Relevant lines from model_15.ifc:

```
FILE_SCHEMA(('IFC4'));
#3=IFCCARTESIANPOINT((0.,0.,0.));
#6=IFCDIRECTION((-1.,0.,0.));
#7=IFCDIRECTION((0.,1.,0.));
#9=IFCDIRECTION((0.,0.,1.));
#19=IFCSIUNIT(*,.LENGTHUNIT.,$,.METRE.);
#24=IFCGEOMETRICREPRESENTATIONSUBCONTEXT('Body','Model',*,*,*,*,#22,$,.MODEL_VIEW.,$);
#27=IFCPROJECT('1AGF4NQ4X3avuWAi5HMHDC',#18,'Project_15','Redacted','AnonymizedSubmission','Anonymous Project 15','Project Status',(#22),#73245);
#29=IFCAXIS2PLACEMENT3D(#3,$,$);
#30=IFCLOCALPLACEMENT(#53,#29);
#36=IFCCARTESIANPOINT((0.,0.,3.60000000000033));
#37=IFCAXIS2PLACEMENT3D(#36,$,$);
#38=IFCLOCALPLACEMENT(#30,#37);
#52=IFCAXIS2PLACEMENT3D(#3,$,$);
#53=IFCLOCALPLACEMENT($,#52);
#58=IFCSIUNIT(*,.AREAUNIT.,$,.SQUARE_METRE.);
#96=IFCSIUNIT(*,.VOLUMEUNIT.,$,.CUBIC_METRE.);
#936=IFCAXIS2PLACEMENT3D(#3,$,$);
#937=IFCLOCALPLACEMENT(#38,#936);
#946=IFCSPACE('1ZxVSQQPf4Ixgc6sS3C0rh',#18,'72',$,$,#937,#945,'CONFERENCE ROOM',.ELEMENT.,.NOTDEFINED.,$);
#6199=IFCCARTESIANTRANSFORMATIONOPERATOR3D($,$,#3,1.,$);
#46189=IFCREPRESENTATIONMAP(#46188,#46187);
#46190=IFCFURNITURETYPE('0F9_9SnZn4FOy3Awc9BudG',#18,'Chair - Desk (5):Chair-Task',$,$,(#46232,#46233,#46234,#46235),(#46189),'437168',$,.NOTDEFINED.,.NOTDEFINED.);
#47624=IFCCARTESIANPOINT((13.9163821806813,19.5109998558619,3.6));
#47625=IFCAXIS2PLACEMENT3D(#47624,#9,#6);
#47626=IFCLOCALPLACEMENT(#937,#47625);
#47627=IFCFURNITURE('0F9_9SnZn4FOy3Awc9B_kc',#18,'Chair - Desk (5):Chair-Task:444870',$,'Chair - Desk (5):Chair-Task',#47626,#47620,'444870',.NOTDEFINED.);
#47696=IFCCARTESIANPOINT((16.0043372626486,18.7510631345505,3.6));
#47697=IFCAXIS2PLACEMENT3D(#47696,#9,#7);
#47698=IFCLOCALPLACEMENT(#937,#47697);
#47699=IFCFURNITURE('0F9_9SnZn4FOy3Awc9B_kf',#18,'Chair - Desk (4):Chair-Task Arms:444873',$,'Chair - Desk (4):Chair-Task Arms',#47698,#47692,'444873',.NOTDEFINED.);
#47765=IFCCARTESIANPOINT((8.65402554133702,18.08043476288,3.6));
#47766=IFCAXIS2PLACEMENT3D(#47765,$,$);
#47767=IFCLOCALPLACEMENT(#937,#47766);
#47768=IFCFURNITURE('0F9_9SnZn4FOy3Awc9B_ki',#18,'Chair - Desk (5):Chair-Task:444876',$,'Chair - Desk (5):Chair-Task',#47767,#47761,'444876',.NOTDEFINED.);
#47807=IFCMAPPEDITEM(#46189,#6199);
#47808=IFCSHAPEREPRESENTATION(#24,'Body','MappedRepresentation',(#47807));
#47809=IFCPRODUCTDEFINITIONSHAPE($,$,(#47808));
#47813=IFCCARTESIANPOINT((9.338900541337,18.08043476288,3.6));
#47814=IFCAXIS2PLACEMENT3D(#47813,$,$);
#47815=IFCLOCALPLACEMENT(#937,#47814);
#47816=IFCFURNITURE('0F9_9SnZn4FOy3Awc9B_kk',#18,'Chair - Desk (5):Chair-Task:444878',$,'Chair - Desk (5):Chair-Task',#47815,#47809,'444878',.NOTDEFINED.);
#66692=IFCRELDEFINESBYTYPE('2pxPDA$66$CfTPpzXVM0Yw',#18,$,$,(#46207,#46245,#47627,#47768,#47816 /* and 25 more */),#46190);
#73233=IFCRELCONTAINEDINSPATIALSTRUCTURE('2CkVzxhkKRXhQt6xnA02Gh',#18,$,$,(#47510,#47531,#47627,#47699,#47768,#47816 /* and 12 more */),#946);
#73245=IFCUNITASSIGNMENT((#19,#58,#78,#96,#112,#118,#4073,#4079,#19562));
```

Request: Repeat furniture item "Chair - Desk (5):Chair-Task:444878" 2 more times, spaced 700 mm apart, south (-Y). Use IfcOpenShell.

```python
import numpy as np
import ifcopenshell
import ifcopenshell.api.geometry
import ifcopenshell.api.root
import ifcopenshell.util.element
import ifcopenshell.util.placement

model = ifcopenshell.open("model_15.ifc")


def reuse_history(source, copy):
    """copy_class also copies each property set's owner history, people and application; keep the originals."""
    for rel in copy.IsDefinedBy:
        if rel.is_a("IfcRelDefinesByProperties") and (history := rel.RelatingPropertyDefinition.OwnerHistory):
            rel.RelatingPropertyDefinition.OwnerHistory = source.OwnerHistory
            ifcopenshell.util.element.remove_deep2(model, history)


source = model.by_guid("0F9_9SnZn4FOy3Awc9B_kk")
base = ifcopenshell.util.placement.get_local_placement(source.ObjectPlacement)
step = np.array([0.0, -1.0, 0.0]) * 0.7

for i in range(1, 3):
    copy = ifcopenshell.api.root.copy_class(model, product=source)
    copy.Representation = ifcopenshell.util.element.copy_deep(
        model, source.Representation, exclude=["IfcGeometricRepresentationContext", "IfcRepresentationMap"]
    )
    copy.Name = "Chair - Desk (5):Chair-Task"
    copy.Tag = None
    reuse_history(source, copy)
    matrix = base.copy()
    matrix[:3, 3] += i * step
    print("added at", matrix[:3, 3].round(3) + 0.0)
    ifcopenshell.api.geometry.edit_object_placement(model, product=copy, matrix=matrix, is_si=False)

model.write("model_15_rev.ifc")
```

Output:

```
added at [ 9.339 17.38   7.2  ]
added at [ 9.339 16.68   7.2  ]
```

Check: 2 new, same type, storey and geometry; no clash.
